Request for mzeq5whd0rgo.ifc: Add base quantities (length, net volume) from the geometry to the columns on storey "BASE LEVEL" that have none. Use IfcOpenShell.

First a look at what the model holds.

```python
import ifcopenshell
import ifcopenshell.util.element
import ifcopenshell.util.unit

model = ifcopenshell.open("mzeq5whd0rgo.ifc")
print(model.schema)
for unit_type in ("LENGTHUNIT", "AREAUNIT", "VOLUMEUNIT"):
    print(unit_type, ifcopenshell.util.unit.calculate_unit_scale(model, unit_type))
storey = next(s for s in model.by_type("IfcBuildingStorey") if s.Name == "BASE LEVEL")
columns = [e for e in ifcopenshell.util.element.get_decomposition(storey) if e.is_a("IfcColumn")]
for e in sorted(columns, key=lambda e: e.id()):
    print(e.id(), e.is_a(), e.Name, list(ifcopenshell.util.element.get_psets(e, qtos_only=True)), sep=" | ")
```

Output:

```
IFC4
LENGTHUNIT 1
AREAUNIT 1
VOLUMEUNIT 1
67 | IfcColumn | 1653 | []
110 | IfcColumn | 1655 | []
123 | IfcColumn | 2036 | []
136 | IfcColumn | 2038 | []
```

```python
import ifcopenshell
import ifcopenshell.api.pset
import ifcopenshell.geom
import ifcopenshell.util.element
import ifcopenshell.util.shape
import ifcopenshell.util.unit

model = ifcopenshell.open("mzeq5whd0rgo.ifc")
unit_scale = ifcopenshell.util.unit.calculate_unit_scale(model)
volume_scale = ifcopenshell.util.unit.calculate_unit_scale(model, "VOLUMEUNIT")
settings = ifcopenshell.geom.settings()

storey = next(s for s in model.by_type("IfcBuildingStorey") if s.Name == "BASE LEVEL")
columns = [e for e in ifcopenshell.util.element.get_decomposition(storey) if e.is_a("IfcColumn")]

for e in sorted(columns, key=lambda e: e.id()):
    if ifcopenshell.util.element.get_psets(e, qtos_only=True, should_inherit=False):
        continue
    # Geometry comes back in metres, in the element's own axes.
    shape = ifcopenshell.geom.create_shape(settings, e)
    values = {
        "Length": ifcopenshell.util.shape.get_z(shape.geometry) / unit_scale,
        "NetVolume": ifcopenshell.util.shape.get_volume(shape.geometry) / volume_scale,
    }
    qto = ifcopenshell.api.pset.add_qto(model, product=e, name="Qto_ColumnBaseQuantities")
    ifcopenshell.api.pset.edit_qto(model, qto=qto, properties=values)
    print(e.id(), {k: round(v, 3) for k, v in values.items()})

model.write("mzeq5whd0rgo_updated.ifc")
```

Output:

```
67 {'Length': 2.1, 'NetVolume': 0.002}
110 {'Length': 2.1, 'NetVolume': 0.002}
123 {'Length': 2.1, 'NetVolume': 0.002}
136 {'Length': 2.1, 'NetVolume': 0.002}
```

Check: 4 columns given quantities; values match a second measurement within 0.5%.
